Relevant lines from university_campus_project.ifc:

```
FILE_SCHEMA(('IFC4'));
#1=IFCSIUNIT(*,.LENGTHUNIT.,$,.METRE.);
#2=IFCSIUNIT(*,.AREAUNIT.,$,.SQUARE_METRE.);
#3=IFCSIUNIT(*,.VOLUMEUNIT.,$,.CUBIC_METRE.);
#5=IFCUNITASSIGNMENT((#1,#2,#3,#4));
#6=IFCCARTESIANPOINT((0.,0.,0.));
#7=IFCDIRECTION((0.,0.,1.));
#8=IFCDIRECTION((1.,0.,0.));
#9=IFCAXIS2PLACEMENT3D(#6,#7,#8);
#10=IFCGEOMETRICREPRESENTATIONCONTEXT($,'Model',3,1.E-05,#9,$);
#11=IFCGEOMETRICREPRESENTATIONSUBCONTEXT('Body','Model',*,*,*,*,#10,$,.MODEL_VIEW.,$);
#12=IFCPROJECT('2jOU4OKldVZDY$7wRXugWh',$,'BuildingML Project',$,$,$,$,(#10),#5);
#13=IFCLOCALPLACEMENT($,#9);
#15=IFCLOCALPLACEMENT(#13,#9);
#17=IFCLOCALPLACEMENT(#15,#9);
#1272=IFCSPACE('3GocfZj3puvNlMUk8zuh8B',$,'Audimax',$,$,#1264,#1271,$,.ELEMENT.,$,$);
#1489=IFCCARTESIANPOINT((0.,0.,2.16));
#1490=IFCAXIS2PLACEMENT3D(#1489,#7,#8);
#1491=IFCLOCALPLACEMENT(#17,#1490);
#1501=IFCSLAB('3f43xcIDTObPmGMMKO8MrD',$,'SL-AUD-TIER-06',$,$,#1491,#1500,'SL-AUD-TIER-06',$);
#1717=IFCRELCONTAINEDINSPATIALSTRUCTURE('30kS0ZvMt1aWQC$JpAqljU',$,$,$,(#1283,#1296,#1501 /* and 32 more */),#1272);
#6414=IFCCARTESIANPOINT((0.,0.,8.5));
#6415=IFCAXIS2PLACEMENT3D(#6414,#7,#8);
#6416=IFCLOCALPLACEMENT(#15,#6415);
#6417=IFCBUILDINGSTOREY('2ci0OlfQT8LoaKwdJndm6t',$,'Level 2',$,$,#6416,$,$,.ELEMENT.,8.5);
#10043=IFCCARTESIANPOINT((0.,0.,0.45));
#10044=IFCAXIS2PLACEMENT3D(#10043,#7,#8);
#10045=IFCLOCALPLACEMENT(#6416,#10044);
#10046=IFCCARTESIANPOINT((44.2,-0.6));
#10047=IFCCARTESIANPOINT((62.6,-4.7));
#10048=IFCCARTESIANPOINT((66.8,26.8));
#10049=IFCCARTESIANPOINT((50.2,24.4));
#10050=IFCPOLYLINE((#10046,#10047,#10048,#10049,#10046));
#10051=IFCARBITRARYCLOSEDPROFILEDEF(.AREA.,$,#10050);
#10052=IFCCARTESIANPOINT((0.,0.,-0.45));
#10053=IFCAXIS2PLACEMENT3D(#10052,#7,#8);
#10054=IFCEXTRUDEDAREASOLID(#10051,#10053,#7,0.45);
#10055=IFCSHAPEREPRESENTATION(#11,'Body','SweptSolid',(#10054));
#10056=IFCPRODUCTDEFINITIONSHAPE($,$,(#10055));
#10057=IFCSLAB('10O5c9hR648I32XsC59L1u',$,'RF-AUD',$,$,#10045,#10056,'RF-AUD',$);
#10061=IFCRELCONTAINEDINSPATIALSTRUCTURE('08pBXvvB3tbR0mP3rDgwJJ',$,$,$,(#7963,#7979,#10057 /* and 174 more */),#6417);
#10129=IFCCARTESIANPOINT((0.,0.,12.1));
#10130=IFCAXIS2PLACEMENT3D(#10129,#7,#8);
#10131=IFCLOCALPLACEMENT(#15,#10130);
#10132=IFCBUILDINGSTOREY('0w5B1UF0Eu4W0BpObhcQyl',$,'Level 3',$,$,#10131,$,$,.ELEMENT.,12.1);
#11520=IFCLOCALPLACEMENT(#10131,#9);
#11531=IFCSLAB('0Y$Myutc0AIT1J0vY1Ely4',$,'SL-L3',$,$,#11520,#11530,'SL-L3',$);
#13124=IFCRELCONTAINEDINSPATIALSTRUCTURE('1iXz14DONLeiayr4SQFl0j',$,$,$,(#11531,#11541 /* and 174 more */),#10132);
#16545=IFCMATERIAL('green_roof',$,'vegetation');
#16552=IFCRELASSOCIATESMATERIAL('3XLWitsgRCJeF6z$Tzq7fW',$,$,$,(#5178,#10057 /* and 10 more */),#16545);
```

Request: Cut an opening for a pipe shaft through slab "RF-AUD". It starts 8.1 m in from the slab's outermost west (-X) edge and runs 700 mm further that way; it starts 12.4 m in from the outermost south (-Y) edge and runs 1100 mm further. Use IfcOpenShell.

```python
import numpy as np
import ifcopenshell
import ifcopenshell.api.feature
import ifcopenshell.api.geometry
import ifcopenshell.api.root
import ifcopenshell.geom
import ifcopenshell.util.placement
import ifcopenshell.util.representation
import ifcopenshell.util.shape
import ifcopenshell.util.unit

model = ifcopenshell.open("university_campus_project.ifc")
unit_scale = ifcopenshell.util.unit.calculate_unit_scale(model)
settings = ifcopenshell.geom.settings()


def volume(element):
    """Net volume in cubic metres, openings subtracted."""
    shape = ifcopenshell.geom.create_shape(settings, element)
    return ifcopenshell.util.shape.get_volume(shape.geometry)


slab = model.by_guid("10O5c9hR648I32XsC59L1u")
before = volume(slab)

# Extent in the slab's own axes, in metres. The edges named are its -X and -Y sides.
slab_shape = ifcopenshell.geom.create_shape(settings, slab)
vertices = ifcopenshell.util.shape.get_vertices(slab_shape.geometry)
x_min, y_min, bottom = vertices.min(axis=0)
top = vertices[:, 2].max()

opening = ifcopenshell.api.root.create_entity(model, ifc_class="IfcOpeningElement", name="Pipe shaft opening", predefined_type="OPENING")
context = ifcopenshell.util.representation.get_context(model, "Model", "Body", "MODEL_VIEW")
width, depth = 0.7, 1.1
outline = [(0.0, 0.0), (width, 0.0), (width, depth), (0.0, depth), (0.0, 0.0)]
# Overshoot both faces by 50 mm so the cut is clean.
shape = ifcopenshell.api.geometry.add_slab_representation(
    model, context=context, depth=top - bottom + 0.1, polyline=outline
)
ifcopenshell.api.geometry.assign_representation(model, product=opening, representation=shape)

matrix = ifcopenshell.util.placement.get_local_placement(slab.ObjectPlacement)
matrix[:, 3] = matrix @ np.append(np.array([x_min + 8.1, y_min + 12.4, bottom - 0.05]) / unit_scale, 1.0)
ifcopenshell.api.geometry.edit_object_placement(model, product=opening, matrix=matrix, is_si=False)
ifcopenshell.api.feature.add_feature(model, feature=opening, element=slab)

after = volume(slab)

print(f"slab volume {before:.3f} -> {after:.3f} m3")

model.write("university_campus_project_v2.ifc")
```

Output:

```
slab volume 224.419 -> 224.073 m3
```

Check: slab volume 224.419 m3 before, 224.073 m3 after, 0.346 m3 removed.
